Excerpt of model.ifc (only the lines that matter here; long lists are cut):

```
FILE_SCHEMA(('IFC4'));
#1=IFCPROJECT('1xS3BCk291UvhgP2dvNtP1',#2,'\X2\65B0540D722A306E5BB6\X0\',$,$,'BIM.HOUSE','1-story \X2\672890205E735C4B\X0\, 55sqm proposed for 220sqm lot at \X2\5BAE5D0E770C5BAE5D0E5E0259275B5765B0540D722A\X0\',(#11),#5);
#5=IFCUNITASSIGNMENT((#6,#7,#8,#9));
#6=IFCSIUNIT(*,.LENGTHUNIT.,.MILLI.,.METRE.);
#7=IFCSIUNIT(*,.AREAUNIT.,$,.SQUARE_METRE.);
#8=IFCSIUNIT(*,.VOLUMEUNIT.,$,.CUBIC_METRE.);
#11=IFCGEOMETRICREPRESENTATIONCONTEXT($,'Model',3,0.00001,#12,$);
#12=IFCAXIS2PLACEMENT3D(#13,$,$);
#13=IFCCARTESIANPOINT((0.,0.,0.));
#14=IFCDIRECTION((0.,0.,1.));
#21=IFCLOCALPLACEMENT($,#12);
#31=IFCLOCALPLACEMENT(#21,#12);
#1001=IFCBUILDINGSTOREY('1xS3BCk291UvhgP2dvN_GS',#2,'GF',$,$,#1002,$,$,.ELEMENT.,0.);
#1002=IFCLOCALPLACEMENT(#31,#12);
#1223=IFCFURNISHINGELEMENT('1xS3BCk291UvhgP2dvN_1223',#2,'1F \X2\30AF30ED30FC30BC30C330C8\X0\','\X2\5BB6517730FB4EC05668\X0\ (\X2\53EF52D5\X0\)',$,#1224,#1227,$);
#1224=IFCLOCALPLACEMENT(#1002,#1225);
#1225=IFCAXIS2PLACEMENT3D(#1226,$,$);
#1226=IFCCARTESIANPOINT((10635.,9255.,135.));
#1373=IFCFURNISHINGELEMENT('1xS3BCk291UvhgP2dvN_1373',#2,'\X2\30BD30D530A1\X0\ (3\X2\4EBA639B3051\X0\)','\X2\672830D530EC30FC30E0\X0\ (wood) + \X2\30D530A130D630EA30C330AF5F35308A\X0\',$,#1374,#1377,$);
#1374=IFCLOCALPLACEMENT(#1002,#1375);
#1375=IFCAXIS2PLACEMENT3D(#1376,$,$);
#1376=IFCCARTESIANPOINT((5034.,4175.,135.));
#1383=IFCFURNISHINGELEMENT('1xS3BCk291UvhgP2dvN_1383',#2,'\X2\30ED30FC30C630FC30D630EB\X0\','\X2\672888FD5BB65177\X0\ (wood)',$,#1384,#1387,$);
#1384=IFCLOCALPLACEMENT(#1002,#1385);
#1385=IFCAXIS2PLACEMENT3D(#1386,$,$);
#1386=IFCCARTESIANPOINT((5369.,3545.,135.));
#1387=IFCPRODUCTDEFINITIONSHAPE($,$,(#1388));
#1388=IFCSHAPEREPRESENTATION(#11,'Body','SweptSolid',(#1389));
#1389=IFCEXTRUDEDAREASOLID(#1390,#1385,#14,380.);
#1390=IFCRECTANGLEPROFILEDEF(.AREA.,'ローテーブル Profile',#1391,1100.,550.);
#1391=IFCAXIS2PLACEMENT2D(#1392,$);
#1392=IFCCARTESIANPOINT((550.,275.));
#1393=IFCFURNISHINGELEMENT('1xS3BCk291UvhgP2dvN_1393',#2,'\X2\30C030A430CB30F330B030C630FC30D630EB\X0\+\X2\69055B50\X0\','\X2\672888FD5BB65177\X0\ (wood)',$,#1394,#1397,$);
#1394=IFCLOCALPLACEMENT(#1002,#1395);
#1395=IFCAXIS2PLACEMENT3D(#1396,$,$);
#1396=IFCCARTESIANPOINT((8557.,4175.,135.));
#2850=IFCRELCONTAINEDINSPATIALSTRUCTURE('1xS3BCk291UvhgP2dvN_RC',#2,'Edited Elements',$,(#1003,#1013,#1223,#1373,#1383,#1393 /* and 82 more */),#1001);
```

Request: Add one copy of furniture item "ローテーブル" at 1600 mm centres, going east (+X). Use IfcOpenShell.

```python
import numpy as np
import ifcopenshell
import ifcopenshell.api.geometry
import ifcopenshell.api.root
import ifcopenshell.util.element
import ifcopenshell.util.placement
import ifcopenshell.util.unit

model = ifcopenshell.open("model.ifc")
unit_scale = ifcopenshell.util.unit.calculate_unit_scale(model)


def reuse_history(source, copy):
    """copy_class also copies each property set's owner history, people and application; keep the originals."""
    for rel in copy.IsDefinedBy:
        if rel.is_a("IfcRelDefinesByProperties") and (history := rel.RelatingPropertyDefinition.OwnerHistory):
            rel.RelatingPropertyDefinition.OwnerHistory = source.OwnerHistory
            ifcopenshell.util.element.remove_deep2(model, history)


source = model.by_guid("1xS3BCk291UvhgP2dvN_1383")
base = ifcopenshell.util.placement.get_local_placement(source.ObjectPlacement)
step = np.array([1.0, 0.0, 0.0]) * 1.6 / unit_scale

for i in range(1, 2):
    copy = ifcopenshell.api.root.copy_class(model, product=source)
    copy.Representation = ifcopenshell.util.element.copy_deep(
        model, source.Representation, exclude=["IfcGeometricRepresentationContext", "IfcRepresentationMap"]
    )
    reuse_history(source, copy)
    matrix = base.copy()
    matrix[:3, 3] += i * step
    print("added at", matrix[:3, 3].round(3) + 0.0)
    ifcopenshell.api.geometry.edit_object_placement(model, product=copy, matrix=matrix, is_si=False)

model.write("model_rev.ifc")
```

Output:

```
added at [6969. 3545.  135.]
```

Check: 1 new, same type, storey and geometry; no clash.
